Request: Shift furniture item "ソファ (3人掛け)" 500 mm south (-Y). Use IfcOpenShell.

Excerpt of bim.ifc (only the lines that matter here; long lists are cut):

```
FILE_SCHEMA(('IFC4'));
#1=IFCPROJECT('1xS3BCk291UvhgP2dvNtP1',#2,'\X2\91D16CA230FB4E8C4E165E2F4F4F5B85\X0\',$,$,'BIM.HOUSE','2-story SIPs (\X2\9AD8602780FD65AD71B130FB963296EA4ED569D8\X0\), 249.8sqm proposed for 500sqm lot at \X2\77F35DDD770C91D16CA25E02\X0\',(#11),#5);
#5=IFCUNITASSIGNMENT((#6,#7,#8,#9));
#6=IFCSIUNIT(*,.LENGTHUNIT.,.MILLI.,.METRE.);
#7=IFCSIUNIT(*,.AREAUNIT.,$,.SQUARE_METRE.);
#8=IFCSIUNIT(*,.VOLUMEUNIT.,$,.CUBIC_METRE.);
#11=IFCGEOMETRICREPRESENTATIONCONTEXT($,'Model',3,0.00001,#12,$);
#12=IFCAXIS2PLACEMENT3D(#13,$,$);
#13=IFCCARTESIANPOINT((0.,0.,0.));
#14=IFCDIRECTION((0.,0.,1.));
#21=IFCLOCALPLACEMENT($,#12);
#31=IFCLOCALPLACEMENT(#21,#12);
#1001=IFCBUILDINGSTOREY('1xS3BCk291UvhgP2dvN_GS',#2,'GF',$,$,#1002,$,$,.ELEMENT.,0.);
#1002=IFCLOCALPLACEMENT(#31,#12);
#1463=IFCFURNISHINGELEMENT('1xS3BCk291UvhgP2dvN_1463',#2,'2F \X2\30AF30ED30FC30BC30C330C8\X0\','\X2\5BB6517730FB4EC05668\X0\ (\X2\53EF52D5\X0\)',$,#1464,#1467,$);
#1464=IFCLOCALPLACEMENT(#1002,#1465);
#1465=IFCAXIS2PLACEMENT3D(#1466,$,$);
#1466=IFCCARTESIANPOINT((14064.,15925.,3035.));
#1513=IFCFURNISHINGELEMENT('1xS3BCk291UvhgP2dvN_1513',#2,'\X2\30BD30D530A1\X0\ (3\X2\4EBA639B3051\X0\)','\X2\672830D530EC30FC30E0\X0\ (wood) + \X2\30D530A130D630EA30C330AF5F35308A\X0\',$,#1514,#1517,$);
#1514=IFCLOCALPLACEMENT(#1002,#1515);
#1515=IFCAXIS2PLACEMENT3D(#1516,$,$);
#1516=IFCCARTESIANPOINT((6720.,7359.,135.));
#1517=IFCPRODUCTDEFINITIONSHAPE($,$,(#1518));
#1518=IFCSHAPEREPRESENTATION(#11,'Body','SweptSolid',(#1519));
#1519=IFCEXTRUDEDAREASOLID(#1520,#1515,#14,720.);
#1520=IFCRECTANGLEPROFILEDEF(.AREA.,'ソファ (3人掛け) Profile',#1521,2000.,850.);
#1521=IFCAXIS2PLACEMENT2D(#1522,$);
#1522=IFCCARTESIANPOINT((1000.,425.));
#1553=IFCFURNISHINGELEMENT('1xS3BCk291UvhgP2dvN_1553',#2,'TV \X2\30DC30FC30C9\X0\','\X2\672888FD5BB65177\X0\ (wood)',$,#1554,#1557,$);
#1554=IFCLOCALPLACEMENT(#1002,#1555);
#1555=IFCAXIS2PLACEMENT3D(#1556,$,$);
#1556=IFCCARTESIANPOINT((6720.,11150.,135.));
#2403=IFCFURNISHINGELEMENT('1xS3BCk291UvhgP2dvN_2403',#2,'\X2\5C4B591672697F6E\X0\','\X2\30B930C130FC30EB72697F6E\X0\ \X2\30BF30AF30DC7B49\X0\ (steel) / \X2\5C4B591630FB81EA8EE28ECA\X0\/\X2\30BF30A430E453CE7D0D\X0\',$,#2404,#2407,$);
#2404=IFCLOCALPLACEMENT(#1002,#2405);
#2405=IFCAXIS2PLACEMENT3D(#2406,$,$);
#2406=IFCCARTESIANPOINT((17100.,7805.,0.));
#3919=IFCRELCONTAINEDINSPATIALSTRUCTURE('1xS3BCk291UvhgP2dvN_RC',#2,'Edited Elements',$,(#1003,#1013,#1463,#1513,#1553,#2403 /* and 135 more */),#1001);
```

```python
import ifcopenshell
import ifcopenshell.api.geometry
import ifcopenshell.util.placement

model = ifcopenshell.open("bim.ifc")

item = model.by_guid("1xS3BCk291UvhgP2dvN_1513")
matrix = ifcopenshell.util.placement.get_local_placement(item.ObjectPlacement)
matrix[1, 3] -= 500.0
ifcopenshell.api.geometry.edit_object_placement(model, product=item, matrix=matrix, is_si=False)

print(ifcopenshell.util.placement.get_local_placement(item.ObjectPlacement).round(3) + 0.0)

model.write("bim_v2.ifc")
```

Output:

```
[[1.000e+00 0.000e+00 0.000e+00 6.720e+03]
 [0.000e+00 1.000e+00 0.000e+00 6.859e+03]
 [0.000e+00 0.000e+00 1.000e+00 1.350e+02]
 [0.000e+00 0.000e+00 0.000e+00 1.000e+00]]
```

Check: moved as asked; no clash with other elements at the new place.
